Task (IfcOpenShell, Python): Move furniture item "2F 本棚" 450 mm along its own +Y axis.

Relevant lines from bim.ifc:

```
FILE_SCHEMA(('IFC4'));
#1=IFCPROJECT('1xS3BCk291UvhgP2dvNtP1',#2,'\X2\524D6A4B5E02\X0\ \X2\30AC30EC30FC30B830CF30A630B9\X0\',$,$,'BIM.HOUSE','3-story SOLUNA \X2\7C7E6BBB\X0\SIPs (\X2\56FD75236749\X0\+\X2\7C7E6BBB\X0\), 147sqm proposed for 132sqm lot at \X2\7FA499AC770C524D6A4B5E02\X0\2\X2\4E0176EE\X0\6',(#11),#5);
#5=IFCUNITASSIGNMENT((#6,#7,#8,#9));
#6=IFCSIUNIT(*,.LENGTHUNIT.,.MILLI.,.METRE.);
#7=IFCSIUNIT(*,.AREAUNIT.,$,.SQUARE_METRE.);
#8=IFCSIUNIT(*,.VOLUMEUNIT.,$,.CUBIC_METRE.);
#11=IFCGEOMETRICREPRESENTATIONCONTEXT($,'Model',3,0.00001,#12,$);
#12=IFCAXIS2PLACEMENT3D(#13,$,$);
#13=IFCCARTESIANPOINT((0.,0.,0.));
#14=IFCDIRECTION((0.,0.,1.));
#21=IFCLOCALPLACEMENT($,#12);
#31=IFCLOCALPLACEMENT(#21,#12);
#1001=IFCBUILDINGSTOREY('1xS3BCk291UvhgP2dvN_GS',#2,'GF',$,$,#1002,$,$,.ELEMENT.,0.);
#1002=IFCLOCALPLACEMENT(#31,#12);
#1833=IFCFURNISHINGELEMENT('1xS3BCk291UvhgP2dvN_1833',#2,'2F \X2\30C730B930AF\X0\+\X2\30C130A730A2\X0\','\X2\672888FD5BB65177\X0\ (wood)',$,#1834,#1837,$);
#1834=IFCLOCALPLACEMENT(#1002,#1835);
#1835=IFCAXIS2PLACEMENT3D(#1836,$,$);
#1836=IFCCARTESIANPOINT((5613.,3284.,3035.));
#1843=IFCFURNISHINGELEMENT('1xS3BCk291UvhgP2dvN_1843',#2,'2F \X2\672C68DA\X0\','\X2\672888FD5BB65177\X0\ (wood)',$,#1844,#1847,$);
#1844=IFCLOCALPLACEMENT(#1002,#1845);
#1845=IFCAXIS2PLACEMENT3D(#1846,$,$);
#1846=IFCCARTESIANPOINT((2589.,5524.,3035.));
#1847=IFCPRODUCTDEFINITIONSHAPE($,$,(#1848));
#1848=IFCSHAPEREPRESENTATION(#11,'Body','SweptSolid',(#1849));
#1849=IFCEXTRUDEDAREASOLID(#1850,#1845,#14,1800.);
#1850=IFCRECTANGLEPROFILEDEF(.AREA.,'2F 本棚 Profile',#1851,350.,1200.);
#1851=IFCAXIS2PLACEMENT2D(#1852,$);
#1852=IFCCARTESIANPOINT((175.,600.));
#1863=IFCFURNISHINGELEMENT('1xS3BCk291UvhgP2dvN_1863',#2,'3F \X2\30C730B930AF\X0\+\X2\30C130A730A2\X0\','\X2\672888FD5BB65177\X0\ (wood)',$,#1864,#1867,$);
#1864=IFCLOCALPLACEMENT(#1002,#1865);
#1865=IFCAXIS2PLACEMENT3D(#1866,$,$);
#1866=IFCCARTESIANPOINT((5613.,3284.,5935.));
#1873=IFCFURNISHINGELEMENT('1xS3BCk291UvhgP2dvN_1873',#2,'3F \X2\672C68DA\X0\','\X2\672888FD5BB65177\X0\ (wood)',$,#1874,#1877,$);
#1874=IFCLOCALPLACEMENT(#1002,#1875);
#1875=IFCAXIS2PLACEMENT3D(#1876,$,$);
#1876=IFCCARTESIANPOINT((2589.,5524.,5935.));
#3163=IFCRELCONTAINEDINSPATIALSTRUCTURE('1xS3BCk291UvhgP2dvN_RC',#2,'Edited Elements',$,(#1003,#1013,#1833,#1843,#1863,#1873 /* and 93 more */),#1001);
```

```python
import ifcopenshell
import ifcopenshell.api.geometry
import ifcopenshell.util.placement

model = ifcopenshell.open("bim.ifc")

item = model.by_guid("1xS3BCk291UvhgP2dvN_1843")
matrix = ifcopenshell.util.placement.get_local_placement(item.ObjectPlacement)
matrix[:3, 3] += matrix[:3, 1] * 450.0
ifcopenshell.api.geometry.edit_object_placement(model, product=item, matrix=matrix, is_si=False)

print(ifcopenshell.util.placement.get_local_placement(item.ObjectPlacement).round(3) + 0.0)

model.write("bim_edited.ifc")
```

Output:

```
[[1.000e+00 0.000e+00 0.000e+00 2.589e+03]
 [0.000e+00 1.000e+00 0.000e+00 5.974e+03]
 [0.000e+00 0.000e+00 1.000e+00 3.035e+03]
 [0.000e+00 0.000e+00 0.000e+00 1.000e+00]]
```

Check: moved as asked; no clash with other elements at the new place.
